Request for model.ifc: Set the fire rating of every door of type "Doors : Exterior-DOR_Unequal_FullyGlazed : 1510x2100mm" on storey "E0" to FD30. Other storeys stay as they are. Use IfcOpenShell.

First a look at what the model holds.

```python
import ifcopenshell
import ifcopenshell.util.element

model = ifcopenshell.open("model.ifc")
print(model.schema)
storey = next(s for s in model.by_type("IfcBuildingStorey") if s.Name == "E0")
doors = [e for e in ifcopenshell.util.element.get_decomposition(storey) if e.is_a("IfcDoor")]
seen = {}
for e in doors:
    element_type = ifcopenshell.util.element.get_type(e)
    key = (element_type.Name if element_type != e and element_type else None, ifcopenshell.util.element.get_pset(e, "Pset_DoorCommon", "FireRating"))
    seen[key] = seen.get(key, 0) + 1
for (name, value), count in sorted(seen.items(), key=str):
    print(count, "x", name, "|", value)
```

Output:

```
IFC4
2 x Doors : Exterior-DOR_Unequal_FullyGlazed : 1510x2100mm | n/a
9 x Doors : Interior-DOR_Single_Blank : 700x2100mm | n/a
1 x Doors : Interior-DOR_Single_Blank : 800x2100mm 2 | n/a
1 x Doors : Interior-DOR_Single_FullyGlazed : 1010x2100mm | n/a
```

```python
import ifcopenshell
import ifcopenshell.api.pset
import ifcopenshell.util.element

model = ifcopenshell.open("model.ifc")

storey = next(s for s in model.by_type("IfcBuildingStorey") if s.Name == "E0")
doors = [e for e in ifcopenshell.util.element.get_decomposition(storey) if e.is_a("IfcDoor")]

count = 0
for e in doors:
    element_type = ifcopenshell.util.element.get_type(e)
    if element_type in (None, e) or element_type.Name != "Doors : Exterior-DOR_Unequal_FullyGlazed : 1510x2100mm":
        continue
    # add_pset returns the element's existing set when there is one.
    pset = ifcopenshell.api.pset.add_pset(model, product=e, name="Pset_DoorCommon")
    ifcopenshell.api.pset.edit_pset(model, pset=pset, properties={"FireRating": "FD30"})
    count += 1

print(count, "doors updated")

model.write("model_v2.ifc")
```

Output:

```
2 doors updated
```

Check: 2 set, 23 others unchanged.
